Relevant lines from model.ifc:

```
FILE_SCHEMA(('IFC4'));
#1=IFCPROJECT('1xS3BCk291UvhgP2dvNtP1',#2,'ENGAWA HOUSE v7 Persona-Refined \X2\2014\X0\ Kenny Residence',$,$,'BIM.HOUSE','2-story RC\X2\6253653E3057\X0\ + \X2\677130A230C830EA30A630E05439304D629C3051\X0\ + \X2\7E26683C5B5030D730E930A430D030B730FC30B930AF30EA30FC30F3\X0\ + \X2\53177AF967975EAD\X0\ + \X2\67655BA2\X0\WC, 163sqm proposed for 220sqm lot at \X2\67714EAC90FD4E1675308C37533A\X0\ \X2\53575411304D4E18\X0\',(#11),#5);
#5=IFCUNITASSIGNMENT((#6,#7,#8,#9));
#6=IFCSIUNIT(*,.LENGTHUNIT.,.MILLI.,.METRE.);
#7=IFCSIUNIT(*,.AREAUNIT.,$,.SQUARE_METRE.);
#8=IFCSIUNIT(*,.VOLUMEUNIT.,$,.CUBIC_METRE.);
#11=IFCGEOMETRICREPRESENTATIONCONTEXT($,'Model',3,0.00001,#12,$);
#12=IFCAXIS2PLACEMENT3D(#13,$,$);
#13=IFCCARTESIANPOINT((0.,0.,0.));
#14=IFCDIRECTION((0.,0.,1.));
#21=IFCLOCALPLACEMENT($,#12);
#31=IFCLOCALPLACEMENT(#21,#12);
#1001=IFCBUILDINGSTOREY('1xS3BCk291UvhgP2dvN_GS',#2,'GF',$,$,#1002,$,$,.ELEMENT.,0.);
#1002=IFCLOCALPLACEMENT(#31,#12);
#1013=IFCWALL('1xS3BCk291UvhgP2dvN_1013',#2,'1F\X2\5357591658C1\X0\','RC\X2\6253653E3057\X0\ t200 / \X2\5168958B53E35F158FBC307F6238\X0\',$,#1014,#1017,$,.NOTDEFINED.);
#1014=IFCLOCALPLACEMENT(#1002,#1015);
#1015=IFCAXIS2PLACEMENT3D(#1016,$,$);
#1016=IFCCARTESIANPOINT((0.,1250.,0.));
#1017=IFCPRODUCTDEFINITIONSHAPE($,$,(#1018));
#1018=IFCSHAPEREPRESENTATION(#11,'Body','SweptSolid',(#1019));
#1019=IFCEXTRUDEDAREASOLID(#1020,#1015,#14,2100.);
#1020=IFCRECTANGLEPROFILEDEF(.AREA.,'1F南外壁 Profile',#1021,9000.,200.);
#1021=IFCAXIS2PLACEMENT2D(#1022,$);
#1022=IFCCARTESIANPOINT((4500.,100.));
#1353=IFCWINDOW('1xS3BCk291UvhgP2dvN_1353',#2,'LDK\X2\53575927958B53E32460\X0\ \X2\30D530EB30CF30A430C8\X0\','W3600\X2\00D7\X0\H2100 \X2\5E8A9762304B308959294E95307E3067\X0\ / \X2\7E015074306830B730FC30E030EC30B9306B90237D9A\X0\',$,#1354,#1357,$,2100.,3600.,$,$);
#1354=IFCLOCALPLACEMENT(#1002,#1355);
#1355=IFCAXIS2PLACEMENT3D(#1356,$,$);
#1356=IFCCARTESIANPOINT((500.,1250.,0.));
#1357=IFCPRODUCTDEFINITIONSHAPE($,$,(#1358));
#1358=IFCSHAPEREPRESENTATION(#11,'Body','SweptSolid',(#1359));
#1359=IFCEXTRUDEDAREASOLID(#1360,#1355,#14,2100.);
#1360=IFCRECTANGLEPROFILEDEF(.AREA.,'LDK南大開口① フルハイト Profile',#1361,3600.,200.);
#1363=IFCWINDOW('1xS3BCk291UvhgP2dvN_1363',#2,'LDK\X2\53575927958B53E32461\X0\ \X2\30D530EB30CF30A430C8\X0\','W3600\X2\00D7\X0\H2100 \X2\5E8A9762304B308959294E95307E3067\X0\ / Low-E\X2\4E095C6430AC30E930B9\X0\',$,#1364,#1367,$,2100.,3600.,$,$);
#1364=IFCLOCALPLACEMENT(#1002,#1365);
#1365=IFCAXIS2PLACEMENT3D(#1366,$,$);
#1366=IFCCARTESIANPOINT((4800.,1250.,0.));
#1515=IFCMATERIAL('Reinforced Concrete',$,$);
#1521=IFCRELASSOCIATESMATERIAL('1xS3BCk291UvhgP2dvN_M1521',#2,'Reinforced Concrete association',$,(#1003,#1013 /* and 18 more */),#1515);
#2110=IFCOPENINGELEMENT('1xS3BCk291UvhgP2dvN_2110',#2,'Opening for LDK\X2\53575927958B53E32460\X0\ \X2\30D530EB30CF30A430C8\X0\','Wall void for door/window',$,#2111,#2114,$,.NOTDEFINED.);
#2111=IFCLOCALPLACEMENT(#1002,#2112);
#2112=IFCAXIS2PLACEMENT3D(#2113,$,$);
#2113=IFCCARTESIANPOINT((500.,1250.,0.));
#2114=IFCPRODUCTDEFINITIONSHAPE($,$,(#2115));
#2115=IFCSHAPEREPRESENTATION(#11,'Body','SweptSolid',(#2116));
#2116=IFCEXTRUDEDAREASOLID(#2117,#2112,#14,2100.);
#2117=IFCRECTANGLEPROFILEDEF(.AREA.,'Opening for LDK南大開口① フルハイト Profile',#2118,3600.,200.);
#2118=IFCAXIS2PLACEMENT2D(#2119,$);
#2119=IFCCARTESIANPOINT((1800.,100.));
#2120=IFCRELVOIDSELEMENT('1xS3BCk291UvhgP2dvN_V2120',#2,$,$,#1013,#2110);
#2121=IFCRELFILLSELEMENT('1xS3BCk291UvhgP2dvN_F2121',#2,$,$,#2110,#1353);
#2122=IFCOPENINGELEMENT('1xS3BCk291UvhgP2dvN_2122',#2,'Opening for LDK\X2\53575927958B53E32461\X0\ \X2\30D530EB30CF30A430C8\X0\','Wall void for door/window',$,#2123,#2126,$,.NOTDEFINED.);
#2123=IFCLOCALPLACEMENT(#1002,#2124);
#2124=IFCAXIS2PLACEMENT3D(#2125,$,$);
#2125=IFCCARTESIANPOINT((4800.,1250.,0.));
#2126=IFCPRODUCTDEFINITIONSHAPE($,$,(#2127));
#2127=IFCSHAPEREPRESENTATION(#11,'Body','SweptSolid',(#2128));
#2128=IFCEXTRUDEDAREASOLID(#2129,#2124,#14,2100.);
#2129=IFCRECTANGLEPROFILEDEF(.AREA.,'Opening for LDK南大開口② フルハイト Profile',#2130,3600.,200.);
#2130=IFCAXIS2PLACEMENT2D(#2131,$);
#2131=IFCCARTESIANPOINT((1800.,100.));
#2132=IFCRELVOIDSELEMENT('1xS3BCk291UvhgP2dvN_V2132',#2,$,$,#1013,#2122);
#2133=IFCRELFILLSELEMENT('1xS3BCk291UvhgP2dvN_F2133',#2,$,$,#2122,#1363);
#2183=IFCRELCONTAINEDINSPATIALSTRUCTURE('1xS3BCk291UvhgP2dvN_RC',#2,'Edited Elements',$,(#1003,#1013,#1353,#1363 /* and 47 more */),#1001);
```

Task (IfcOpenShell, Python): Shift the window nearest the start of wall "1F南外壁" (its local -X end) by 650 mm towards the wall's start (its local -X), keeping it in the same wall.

```python
import ifcopenshell
import ifcopenshell.api.geometry
import ifcopenshell.util.placement
import ifcopenshell.util.unit

model = ifcopenshell.open("model.ifc")
unit_scale = ifcopenshell.util.unit.calculate_unit_scale(model)

window = model.by_guid("1xS3BCk291UvhgP2dvN_1353")
opening = window.FillsVoids[0].RelatingOpeningElement
wall = opening.VoidsElements[0].RelatingBuildingElement

wall_matrix = ifcopenshell.util.placement.get_local_placement(wall.ObjectPlacement)
shift = wall_matrix[:3, 0] * -0.65 / unit_scale
before = ifcopenshell.util.placement.get_local_placement(window.ObjectPlacement)[:3, 3].copy()

# The window is not placed relative to its opening, so move both.
for product in (opening, window):
    matrix = ifcopenshell.util.placement.get_local_placement(product.ObjectPlacement)
    matrix[:3, 3] += shift
    ifcopenshell.api.geometry.edit_object_placement(model, product=product, matrix=matrix, is_si=False)

after = ifcopenshell.util.placement.get_local_placement(window.ObjectPlacement)[:3, 3]
print("window moved by", (after - before).round(3) + 0.0)

model.write("model_edited.ifc")
```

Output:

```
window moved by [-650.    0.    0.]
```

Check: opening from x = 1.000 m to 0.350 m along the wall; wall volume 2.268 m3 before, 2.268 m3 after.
